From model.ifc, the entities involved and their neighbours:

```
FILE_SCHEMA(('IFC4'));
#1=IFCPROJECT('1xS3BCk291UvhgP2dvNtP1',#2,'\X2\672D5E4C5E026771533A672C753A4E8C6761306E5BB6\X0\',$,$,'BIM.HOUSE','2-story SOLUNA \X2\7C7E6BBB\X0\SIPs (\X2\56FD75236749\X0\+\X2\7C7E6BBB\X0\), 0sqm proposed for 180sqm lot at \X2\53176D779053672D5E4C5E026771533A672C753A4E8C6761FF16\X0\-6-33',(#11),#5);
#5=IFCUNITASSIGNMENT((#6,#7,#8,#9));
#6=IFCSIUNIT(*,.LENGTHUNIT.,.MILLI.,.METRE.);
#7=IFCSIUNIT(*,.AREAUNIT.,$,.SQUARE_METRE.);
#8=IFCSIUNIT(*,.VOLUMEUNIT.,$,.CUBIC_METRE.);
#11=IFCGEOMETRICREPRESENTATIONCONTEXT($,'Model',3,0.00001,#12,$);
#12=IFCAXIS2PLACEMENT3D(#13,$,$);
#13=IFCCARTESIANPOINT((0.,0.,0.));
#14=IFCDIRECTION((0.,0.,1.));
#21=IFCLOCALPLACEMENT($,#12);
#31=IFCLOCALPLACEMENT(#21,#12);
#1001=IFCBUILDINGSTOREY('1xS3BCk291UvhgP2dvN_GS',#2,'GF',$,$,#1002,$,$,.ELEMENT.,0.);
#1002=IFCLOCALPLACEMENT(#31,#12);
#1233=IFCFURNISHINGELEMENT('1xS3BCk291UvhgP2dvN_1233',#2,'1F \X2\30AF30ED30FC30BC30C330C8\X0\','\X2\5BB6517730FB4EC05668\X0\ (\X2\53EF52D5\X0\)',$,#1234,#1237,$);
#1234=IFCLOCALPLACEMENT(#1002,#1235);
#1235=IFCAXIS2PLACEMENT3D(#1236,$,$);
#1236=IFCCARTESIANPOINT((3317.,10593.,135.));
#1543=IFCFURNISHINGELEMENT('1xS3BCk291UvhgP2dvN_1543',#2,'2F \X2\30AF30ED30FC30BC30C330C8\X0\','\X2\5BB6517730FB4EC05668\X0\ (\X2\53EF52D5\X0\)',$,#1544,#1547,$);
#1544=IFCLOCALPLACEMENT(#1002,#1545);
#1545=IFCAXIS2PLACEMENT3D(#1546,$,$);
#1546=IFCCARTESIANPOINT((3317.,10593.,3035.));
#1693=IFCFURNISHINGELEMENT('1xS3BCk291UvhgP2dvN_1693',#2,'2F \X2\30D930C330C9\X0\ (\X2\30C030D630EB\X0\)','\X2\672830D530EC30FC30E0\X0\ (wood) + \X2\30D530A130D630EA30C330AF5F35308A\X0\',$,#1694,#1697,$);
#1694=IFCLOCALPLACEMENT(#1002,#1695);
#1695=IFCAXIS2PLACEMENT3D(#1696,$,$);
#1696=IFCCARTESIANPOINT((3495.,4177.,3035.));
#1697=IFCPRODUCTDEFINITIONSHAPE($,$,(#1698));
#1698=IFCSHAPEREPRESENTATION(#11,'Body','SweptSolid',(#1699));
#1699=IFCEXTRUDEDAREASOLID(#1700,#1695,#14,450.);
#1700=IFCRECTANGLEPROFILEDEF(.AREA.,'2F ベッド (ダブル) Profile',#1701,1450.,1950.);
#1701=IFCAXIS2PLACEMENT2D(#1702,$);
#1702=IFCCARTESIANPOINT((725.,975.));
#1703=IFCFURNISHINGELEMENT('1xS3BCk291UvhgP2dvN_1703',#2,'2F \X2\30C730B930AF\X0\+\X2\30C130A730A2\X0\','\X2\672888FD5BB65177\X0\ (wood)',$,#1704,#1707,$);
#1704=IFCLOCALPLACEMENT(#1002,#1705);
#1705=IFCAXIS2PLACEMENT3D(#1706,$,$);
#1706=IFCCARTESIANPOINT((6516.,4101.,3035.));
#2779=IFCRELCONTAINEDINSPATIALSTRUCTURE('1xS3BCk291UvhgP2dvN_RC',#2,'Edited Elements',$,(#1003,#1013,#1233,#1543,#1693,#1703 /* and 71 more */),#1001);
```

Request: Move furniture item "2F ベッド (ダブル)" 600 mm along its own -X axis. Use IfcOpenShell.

```python
import ifcopenshell
import ifcopenshell.api.geometry
import ifcopenshell.util.placement
import ifcopenshell.util.unit

model = ifcopenshell.open("model.ifc")
unit_scale = ifcopenshell.util.unit.calculate_unit_scale(model)

item = model.by_id(1693)
matrix = ifcopenshell.util.placement.get_local_placement(item.ObjectPlacement)
matrix[:3, 3] -= matrix[:3, 0] * 0.6 / unit_scale
ifcopenshell.api.geometry.edit_object_placement(model, product=item, matrix=matrix, is_si=False)

print(ifcopenshell.util.placement.get_local_placement(item.ObjectPlacement).round(3) + 0.0)

model.write("model_rev.ifc")
```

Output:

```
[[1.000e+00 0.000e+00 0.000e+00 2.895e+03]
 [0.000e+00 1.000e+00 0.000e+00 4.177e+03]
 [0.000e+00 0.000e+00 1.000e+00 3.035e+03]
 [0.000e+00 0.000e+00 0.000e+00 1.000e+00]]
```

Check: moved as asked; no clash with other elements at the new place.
